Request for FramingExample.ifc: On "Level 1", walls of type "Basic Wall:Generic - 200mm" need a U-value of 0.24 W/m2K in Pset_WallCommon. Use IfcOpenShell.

First a look at what the model holds.

```python
import ifcopenshell
import ifcopenshell.util.element

model = ifcopenshell.open("FramingExample.ifc")
print(model.schema)
storey = next(s for s in model.by_type("IfcBuildingStorey") if s.Name == "Level 1")
walls = [e for e in ifcopenshell.util.element.get_decomposition(storey) if e.is_a("IfcWall")]
seen = {}
for e in walls:
    element_type = ifcopenshell.util.element.get_type(e)
    key = (element_type.Name if element_type != e and element_type else None, ifcopenshell.util.element.get_pset(e, "Pset_WallCommon", "ThermalTransmittance"))
    seen[key] = seen.get(key, 0) + 1
for (name, value), count in sorted(seen.items(), key=str):
    print(count, "x", name, "|", value)
```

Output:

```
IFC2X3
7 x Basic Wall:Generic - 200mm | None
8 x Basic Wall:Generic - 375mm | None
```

```python
import ifcopenshell
import ifcopenshell.api.pset
import ifcopenshell.util.element

model = ifcopenshell.open("FramingExample.ifc")

storey = next(s for s in model.by_type("IfcBuildingStorey") if s.Name == "Level 1")
walls = [e for e in ifcopenshell.util.element.get_decomposition(storey) if e.is_a("IfcWall")]

count = 0
for e in walls:
    element_type = ifcopenshell.util.element.get_type(e)
    if element_type in (None, e) or element_type.Name != "Basic Wall:Generic - 200mm":
        continue
    # add_pset returns the element's existing set when there is one.
    pset = ifcopenshell.api.pset.add_pset(model, product=e, name="Pset_WallCommon")
    ifcopenshell.api.pset.edit_pset(model, pset=pset, properties={"ThermalTransmittance": 0.24})
    count += 1

print(count, "walls updated")

model.write("FramingExample-out.ifc")
```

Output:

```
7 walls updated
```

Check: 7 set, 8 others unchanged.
